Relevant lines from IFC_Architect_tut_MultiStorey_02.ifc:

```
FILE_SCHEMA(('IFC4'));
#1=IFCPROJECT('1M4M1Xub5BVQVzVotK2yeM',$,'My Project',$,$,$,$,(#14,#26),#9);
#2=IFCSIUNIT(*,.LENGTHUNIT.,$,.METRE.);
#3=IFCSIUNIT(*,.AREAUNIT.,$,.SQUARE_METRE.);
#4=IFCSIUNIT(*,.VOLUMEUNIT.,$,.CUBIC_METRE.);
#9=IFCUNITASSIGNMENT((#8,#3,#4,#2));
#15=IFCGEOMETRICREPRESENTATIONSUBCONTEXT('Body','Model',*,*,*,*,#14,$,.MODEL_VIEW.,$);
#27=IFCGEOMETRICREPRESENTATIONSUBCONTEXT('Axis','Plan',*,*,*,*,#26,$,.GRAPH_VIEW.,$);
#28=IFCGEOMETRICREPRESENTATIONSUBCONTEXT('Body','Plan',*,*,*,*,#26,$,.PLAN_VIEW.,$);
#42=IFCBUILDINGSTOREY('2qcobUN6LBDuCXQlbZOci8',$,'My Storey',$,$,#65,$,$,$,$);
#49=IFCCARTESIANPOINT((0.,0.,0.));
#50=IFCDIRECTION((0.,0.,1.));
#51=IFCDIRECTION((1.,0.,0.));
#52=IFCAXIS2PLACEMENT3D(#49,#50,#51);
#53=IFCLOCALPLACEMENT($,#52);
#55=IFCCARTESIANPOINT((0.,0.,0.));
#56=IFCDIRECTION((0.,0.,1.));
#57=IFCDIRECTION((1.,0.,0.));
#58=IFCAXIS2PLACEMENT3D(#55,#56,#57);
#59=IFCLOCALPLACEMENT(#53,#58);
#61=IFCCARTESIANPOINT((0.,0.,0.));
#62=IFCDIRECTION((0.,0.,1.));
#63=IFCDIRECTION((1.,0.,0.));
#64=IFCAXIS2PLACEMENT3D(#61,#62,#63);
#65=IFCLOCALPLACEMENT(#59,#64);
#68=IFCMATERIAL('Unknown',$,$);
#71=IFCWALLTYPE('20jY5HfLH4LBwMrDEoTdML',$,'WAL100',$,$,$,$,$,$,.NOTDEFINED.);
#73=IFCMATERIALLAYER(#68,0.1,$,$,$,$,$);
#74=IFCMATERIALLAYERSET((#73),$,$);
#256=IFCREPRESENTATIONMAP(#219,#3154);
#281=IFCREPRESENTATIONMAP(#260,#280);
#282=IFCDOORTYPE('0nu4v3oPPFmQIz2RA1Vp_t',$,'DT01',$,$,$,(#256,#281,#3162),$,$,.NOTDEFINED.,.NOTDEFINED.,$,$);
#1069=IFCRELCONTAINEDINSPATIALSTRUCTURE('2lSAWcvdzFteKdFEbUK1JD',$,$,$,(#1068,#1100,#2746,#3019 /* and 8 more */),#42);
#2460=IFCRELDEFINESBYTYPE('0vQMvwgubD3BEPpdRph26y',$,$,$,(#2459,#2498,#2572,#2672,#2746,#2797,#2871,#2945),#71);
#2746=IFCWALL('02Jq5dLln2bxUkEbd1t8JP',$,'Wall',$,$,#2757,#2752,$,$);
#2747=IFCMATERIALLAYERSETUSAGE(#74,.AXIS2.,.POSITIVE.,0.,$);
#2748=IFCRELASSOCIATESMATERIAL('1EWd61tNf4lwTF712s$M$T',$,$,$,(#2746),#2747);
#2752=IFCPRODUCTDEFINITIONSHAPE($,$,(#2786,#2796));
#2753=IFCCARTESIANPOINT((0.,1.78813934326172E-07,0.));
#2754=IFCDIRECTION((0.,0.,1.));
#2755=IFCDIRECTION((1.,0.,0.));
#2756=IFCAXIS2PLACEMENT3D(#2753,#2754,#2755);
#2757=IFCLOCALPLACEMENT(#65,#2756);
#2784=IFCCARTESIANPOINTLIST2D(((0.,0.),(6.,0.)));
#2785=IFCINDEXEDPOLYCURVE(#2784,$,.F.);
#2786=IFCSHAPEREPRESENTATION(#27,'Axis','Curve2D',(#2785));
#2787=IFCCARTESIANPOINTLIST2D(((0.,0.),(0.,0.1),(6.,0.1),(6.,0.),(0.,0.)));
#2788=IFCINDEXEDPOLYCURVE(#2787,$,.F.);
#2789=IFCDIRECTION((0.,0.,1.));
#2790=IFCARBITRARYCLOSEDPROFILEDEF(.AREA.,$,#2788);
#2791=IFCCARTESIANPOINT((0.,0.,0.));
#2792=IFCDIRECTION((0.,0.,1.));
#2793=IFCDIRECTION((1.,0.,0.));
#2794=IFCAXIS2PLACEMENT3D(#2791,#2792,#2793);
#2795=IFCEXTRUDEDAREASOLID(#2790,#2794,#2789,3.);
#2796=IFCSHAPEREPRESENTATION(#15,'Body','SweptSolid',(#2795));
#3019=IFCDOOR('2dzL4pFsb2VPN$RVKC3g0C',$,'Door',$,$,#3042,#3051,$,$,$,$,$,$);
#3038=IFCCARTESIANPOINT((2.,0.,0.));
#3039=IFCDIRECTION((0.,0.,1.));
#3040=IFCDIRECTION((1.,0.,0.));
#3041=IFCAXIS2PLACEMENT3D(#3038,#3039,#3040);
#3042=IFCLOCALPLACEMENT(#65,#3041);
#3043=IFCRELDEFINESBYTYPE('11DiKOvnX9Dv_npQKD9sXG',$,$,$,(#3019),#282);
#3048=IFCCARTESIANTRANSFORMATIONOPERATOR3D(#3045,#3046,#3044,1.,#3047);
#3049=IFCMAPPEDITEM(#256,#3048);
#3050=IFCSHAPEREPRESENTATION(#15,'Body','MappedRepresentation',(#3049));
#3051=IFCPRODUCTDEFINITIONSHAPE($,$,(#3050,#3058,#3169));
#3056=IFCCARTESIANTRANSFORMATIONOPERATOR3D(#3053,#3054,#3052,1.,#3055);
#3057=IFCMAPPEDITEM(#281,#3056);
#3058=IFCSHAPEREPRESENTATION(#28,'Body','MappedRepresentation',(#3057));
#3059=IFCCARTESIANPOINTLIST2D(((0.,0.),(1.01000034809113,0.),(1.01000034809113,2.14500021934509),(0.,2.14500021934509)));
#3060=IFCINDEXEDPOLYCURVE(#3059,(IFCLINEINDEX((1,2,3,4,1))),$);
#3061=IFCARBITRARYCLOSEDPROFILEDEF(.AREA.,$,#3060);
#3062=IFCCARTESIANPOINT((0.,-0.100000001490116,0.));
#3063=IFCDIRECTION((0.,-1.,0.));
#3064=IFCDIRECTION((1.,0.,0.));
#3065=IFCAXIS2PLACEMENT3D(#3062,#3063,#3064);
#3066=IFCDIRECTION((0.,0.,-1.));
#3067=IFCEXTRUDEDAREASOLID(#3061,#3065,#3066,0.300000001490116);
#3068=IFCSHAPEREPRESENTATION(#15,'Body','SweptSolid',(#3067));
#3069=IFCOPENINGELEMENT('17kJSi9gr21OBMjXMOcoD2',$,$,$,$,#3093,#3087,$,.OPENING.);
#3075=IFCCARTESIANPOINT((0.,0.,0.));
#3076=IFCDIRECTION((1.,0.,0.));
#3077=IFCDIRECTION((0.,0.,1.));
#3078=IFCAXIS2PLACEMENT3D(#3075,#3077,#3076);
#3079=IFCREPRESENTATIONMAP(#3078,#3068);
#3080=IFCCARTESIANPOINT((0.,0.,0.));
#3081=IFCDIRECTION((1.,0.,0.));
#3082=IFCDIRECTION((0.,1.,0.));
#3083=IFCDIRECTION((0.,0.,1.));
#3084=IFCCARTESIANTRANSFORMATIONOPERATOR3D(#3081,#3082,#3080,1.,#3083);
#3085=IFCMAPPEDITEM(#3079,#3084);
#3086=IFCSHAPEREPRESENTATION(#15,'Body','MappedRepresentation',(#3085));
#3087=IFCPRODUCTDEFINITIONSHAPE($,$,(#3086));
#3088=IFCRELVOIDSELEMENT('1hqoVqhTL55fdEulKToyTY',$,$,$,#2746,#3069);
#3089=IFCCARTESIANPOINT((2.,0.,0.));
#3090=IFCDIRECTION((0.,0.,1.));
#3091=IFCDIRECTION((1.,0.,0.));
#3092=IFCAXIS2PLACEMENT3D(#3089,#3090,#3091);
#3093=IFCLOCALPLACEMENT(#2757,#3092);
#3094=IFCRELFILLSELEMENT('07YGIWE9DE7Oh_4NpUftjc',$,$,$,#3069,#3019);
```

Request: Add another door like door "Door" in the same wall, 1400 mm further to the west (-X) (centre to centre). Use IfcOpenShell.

```python
import ifcopenshell
import ifcopenshell.api.feature
import ifcopenshell.api.geometry
import ifcopenshell.api.root
import ifcopenshell.geom
import ifcopenshell.util.element
import ifcopenshell.util.placement
import ifcopenshell.util.shape

model = ifcopenshell.open("IFC_Architect_tut_MultiStorey_02.ifc")
settings = ifcopenshell.geom.settings()


def volume(element):
    """Net volume in cubic metres, openings subtracted."""
    shape = ifcopenshell.geom.create_shape(settings, element)
    return ifcopenshell.util.shape.get_volume(shape.geometry)


door = model.by_id(3019)
opening = door.FillsVoids[0].RelatingOpeningElement
wall = opening.VoidsElements[0].RelatingBuildingElement
before = volume(wall)
shift = ifcopenshell.util.placement.get_local_placement(wall.ObjectPlacement)[:3, 0] * -1.4

# copy_class copies the void relationship, type, container and properties, but no geometry.
new_opening = ifcopenshell.api.root.copy_class(model, product=opening)
new_opening.Representation = ifcopenshell.util.element.copy_deep(
    model, opening.Representation, exclude=["IfcGeometricRepresentationContext", "IfcRepresentationMap"]
)
new_door = ifcopenshell.api.root.copy_class(model, product=door)
new_door.Representation = ifcopenshell.util.element.copy_deep(
    model, door.Representation, exclude=["IfcGeometricRepresentationContext", "IfcRepresentationMap"]
)
ifcopenshell.api.feature.add_filling(model, opening=new_opening, element=new_door)

for old, new in ((opening, new_opening), (door, new_door)):
    matrix = ifcopenshell.util.placement.get_local_placement(old.ObjectPlacement)
    matrix[:3, 3] += shift
    ifcopenshell.api.geometry.edit_object_placement(model, product=new, matrix=matrix, is_si=False)

after = volume(wall)

print(f"wall volume {before:.3f} -> {after:.3f} m3")

model.write("IFC_Architect_tut_MultiStorey_02_rev.ifc")
```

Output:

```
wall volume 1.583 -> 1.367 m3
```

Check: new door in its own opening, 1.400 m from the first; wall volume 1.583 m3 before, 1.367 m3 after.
